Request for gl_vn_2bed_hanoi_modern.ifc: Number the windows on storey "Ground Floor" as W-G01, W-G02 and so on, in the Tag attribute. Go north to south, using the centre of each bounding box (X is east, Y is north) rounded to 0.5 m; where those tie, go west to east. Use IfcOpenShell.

First a look at what the model holds.

```python
import ifcopenshell
import ifcopenshell.util.element
import ifcopenshell.util.placement

model = ifcopenshell.open("gl_vn_2bed_hanoi_modern.ifc")
print(model.schema)
storey = next(s for s in model.by_type("IfcBuildingStorey") if s.Name == "Ground Floor")
windows = [e for e in ifcopenshell.util.element.get_decomposition(storey) if e.is_a("IfcWindow")]
for e in sorted(windows, key=lambda e: e.id()):
    origin = ifcopenshell.util.placement.get_local_placement(e.ObjectPlacement)[:3, 3]
    print(e.id(), e.Tag, e.Name, origin.round(2) + 0.0, sep=" | ")
```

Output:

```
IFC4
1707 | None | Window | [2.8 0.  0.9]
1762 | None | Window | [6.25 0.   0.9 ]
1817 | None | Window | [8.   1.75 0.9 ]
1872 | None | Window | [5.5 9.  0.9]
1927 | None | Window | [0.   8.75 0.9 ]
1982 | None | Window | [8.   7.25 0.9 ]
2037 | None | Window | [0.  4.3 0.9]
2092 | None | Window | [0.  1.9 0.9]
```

```python
import ifcopenshell
import ifcopenshell.geom
import ifcopenshell.util.element
import ifcopenshell.util.shape

model = ifcopenshell.open("gl_vn_2bed_hanoi_modern.ifc")
settings = ifcopenshell.geom.settings()
settings.set("use-world-coords", True)


def centre(element):
    shape = ifcopenshell.geom.create_shape(settings, element)
    return ifcopenshell.util.shape.get_bbox_centroid(shape.geometry)


storey = next(s for s in model.by_type("IfcBuildingStorey") if s.Name == "Ground Floor")
windows = [e for e in ifcopenshell.util.element.get_decomposition(storey) if e.is_a("IfcWindow")]

# Insertion points can sit at a corner or the storey origin, so sort by the geometry (in metres).
centres = {e: centre(e) for e in windows}
windows.sort(key=lambda e: (-round(centres[e][1] / 0.5), centres[e][0]))

for i, e in enumerate(windows, start=1):
    number = f"W-G{i:02d}"
    e.Tag = number
    print(e.id(), number)

model.write("gl_vn_2bed_hanoi_modern-out.ifc")
```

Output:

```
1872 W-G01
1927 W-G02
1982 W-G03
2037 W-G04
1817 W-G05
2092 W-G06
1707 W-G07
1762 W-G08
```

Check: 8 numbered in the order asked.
